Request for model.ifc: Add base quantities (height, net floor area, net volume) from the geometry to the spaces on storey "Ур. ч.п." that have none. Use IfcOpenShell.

First a look at what the model holds.

```python
import ifcopenshell
import ifcopenshell.util.element
import ifcopenshell.util.unit

model = ifcopenshell.open("model.ifc")
print(model.schema)
for unit_type in ("LENGTHUNIT", "AREAUNIT", "VOLUMEUNIT"):
    print(unit_type, ifcopenshell.util.unit.calculate_unit_scale(model, unit_type))
storey = next(s for s in model.by_type("IfcBuildingStorey") if s.Name == "Ур. ч.п.")
spaces = [e for e in ifcopenshell.util.element.get_decomposition(storey) if e.is_a("IfcSpace")]
for e in sorted(spaces, key=lambda e: e.id()):
    print(e.id(), e.is_a(), e.Name, list(ifcopenshell.util.element.get_psets(e, qtos_only=True)), sep=" | ")
```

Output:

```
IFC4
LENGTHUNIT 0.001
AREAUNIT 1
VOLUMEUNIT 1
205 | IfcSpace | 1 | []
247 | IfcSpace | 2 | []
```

```python
import ifcopenshell
import ifcopenshell.api.pset
import ifcopenshell.geom
import ifcopenshell.util.element
import ifcopenshell.util.shape
import ifcopenshell.util.unit

model = ifcopenshell.open("model.ifc")
unit_scale = ifcopenshell.util.unit.calculate_unit_scale(model)
area_scale = ifcopenshell.util.unit.calculate_unit_scale(model, "AREAUNIT")
volume_scale = ifcopenshell.util.unit.calculate_unit_scale(model, "VOLUMEUNIT")
settings = ifcopenshell.geom.settings()

storey = next(s for s in model.by_type("IfcBuildingStorey") if s.Name == "Ур. ч.п.")
spaces = [e for e in ifcopenshell.util.element.get_decomposition(storey) if e.is_a("IfcSpace")]

for e in sorted(spaces, key=lambda e: e.id()):
    if ifcopenshell.util.element.get_psets(e, qtos_only=True, should_inherit=False):
        continue
    # Geometry comes back in metres, in the element's own axes.
    shape = ifcopenshell.geom.create_shape(settings, e)
    values = {
        "Height": ifcopenshell.util.shape.get_z(shape.geometry) / unit_scale,
        "NetFloorArea": ifcopenshell.util.shape.get_footprint_area(shape.geometry) / area_scale,
        "NetVolume": ifcopenshell.util.shape.get_volume(shape.geometry) / volume_scale,
    }
    qto = ifcopenshell.api.pset.add_qto(model, product=e, name="Qto_SpaceBaseQuantities")
    ifcopenshell.api.pset.edit_qto(model, qto=qto, properties=values)
    print(e.id(), {k: round(v, 3) for k, v in values.items()})

model.write("model_rev.ifc")
```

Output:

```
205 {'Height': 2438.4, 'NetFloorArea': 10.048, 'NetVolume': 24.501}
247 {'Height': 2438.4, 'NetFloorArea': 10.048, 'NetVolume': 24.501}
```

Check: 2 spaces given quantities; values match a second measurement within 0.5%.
